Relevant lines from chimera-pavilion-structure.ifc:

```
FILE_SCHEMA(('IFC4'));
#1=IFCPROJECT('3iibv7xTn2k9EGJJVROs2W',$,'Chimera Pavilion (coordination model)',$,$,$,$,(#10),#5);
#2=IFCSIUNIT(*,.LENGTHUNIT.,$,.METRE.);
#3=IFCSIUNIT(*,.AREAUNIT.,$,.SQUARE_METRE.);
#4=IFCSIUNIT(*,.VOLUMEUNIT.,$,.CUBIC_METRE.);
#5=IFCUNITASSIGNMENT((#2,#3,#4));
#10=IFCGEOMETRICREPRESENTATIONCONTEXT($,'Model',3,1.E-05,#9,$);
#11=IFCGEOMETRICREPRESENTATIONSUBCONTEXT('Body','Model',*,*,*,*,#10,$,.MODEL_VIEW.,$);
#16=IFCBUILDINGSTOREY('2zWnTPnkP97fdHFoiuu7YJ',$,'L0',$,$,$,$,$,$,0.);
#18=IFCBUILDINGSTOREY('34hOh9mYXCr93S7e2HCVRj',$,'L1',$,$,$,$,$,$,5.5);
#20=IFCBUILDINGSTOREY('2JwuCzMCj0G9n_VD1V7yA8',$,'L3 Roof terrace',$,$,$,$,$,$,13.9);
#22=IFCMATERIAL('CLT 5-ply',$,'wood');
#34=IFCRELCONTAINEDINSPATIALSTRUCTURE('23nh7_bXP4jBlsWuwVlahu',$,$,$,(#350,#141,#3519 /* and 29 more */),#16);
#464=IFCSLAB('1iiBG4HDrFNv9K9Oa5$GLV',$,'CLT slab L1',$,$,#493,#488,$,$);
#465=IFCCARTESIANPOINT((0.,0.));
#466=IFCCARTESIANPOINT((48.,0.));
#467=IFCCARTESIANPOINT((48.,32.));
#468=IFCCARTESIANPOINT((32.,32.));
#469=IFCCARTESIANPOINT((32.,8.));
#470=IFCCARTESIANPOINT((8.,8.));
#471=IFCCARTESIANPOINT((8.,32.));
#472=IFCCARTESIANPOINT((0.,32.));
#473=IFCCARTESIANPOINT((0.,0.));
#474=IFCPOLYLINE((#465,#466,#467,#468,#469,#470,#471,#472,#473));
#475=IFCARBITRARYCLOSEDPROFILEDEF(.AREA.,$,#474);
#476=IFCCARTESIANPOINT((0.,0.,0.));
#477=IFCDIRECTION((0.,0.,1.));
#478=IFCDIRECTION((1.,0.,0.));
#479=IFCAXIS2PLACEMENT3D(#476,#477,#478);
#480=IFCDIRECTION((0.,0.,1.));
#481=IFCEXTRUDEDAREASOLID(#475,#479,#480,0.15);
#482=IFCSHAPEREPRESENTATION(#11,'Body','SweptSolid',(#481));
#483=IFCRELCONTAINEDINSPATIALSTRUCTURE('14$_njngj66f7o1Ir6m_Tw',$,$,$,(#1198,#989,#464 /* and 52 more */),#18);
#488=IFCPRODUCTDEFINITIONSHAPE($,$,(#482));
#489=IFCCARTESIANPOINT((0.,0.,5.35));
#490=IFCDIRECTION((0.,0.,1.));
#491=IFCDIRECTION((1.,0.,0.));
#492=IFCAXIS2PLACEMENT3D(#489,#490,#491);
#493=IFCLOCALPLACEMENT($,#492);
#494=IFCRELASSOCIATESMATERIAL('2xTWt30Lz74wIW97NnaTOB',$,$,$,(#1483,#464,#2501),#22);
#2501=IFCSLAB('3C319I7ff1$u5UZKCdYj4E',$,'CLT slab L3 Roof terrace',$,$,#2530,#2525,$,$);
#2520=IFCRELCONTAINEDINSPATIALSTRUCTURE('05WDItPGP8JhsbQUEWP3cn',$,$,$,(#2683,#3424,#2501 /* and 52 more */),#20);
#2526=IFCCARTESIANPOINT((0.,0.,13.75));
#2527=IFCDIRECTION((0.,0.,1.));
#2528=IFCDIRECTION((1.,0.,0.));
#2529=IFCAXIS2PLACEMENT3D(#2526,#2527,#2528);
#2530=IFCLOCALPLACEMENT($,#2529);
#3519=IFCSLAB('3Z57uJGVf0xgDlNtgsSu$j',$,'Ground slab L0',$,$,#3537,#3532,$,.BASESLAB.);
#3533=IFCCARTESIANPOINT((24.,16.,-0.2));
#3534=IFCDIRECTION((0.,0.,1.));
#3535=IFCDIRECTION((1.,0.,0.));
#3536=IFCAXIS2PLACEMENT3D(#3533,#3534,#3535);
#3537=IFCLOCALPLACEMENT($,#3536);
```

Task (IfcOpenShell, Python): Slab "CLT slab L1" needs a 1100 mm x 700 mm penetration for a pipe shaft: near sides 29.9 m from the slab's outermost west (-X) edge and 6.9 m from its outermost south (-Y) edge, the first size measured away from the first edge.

```python
import numpy as np
import ifcopenshell
import ifcopenshell.api.feature
import ifcopenshell.api.geometry
import ifcopenshell.api.root
import ifcopenshell.geom
import ifcopenshell.util.placement
import ifcopenshell.util.representation
import ifcopenshell.util.shape
import ifcopenshell.util.unit

model = ifcopenshell.open("chimera-pavilion-structure.ifc")
unit_scale = ifcopenshell.util.unit.calculate_unit_scale(model)
settings = ifcopenshell.geom.settings()


def volume(element):
    """Net volume in cubic metres, openings subtracted."""
    shape = ifcopenshell.geom.create_shape(settings, element)
    return ifcopenshell.util.shape.get_volume(shape.geometry)


slab = model.by_guid("1iiBG4HDrFNv9K9Oa5$GLV")
before = volume(slab)

# Extent in the slab's own axes, in metres. The edges named are its -X and -Y sides.
slab_shape = ifcopenshell.geom.create_shape(settings, slab)
vertices = ifcopenshell.util.shape.get_vertices(slab_shape.geometry)
x_min, y_min, bottom = vertices.min(axis=0)
top = vertices[:, 2].max()

opening = ifcopenshell.api.root.create_entity(model, ifc_class="IfcOpeningElement", name="Pipe shaft opening", predefined_type="OPENING")
context = ifcopenshell.util.representation.get_context(model, "Model", "Body", "MODEL_VIEW")
width, depth = 1.1, 0.7
outline = [(0.0, 0.0), (width, 0.0), (width, depth), (0.0, depth), (0.0, 0.0)]
# Overshoot both faces by 50 mm so the cut is clean.
shape = ifcopenshell.api.geometry.add_slab_representation(
    model, context=context, depth=top - bottom + 0.1, polyline=outline
)
ifcopenshell.api.geometry.assign_representation(model, product=opening, representation=shape)

matrix = ifcopenshell.util.placement.get_local_placement(slab.ObjectPlacement)
matrix[:, 3] = matrix @ np.append(np.array([x_min + 29.9, y_min + 6.9, bottom - 0.05]) / unit_scale, 1.0)
ifcopenshell.api.geometry.edit_object_placement(model, product=opening, matrix=matrix, is_si=False)
ifcopenshell.api.feature.add_feature(model, feature=opening, element=slab)

after = volume(slab)

print(f"slab volume {before:.3f} -> {after:.3f} m3")

model.write("chimera-pavilion-structure_v2.ifc")
```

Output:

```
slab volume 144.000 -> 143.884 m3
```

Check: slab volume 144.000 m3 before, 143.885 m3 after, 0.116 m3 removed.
